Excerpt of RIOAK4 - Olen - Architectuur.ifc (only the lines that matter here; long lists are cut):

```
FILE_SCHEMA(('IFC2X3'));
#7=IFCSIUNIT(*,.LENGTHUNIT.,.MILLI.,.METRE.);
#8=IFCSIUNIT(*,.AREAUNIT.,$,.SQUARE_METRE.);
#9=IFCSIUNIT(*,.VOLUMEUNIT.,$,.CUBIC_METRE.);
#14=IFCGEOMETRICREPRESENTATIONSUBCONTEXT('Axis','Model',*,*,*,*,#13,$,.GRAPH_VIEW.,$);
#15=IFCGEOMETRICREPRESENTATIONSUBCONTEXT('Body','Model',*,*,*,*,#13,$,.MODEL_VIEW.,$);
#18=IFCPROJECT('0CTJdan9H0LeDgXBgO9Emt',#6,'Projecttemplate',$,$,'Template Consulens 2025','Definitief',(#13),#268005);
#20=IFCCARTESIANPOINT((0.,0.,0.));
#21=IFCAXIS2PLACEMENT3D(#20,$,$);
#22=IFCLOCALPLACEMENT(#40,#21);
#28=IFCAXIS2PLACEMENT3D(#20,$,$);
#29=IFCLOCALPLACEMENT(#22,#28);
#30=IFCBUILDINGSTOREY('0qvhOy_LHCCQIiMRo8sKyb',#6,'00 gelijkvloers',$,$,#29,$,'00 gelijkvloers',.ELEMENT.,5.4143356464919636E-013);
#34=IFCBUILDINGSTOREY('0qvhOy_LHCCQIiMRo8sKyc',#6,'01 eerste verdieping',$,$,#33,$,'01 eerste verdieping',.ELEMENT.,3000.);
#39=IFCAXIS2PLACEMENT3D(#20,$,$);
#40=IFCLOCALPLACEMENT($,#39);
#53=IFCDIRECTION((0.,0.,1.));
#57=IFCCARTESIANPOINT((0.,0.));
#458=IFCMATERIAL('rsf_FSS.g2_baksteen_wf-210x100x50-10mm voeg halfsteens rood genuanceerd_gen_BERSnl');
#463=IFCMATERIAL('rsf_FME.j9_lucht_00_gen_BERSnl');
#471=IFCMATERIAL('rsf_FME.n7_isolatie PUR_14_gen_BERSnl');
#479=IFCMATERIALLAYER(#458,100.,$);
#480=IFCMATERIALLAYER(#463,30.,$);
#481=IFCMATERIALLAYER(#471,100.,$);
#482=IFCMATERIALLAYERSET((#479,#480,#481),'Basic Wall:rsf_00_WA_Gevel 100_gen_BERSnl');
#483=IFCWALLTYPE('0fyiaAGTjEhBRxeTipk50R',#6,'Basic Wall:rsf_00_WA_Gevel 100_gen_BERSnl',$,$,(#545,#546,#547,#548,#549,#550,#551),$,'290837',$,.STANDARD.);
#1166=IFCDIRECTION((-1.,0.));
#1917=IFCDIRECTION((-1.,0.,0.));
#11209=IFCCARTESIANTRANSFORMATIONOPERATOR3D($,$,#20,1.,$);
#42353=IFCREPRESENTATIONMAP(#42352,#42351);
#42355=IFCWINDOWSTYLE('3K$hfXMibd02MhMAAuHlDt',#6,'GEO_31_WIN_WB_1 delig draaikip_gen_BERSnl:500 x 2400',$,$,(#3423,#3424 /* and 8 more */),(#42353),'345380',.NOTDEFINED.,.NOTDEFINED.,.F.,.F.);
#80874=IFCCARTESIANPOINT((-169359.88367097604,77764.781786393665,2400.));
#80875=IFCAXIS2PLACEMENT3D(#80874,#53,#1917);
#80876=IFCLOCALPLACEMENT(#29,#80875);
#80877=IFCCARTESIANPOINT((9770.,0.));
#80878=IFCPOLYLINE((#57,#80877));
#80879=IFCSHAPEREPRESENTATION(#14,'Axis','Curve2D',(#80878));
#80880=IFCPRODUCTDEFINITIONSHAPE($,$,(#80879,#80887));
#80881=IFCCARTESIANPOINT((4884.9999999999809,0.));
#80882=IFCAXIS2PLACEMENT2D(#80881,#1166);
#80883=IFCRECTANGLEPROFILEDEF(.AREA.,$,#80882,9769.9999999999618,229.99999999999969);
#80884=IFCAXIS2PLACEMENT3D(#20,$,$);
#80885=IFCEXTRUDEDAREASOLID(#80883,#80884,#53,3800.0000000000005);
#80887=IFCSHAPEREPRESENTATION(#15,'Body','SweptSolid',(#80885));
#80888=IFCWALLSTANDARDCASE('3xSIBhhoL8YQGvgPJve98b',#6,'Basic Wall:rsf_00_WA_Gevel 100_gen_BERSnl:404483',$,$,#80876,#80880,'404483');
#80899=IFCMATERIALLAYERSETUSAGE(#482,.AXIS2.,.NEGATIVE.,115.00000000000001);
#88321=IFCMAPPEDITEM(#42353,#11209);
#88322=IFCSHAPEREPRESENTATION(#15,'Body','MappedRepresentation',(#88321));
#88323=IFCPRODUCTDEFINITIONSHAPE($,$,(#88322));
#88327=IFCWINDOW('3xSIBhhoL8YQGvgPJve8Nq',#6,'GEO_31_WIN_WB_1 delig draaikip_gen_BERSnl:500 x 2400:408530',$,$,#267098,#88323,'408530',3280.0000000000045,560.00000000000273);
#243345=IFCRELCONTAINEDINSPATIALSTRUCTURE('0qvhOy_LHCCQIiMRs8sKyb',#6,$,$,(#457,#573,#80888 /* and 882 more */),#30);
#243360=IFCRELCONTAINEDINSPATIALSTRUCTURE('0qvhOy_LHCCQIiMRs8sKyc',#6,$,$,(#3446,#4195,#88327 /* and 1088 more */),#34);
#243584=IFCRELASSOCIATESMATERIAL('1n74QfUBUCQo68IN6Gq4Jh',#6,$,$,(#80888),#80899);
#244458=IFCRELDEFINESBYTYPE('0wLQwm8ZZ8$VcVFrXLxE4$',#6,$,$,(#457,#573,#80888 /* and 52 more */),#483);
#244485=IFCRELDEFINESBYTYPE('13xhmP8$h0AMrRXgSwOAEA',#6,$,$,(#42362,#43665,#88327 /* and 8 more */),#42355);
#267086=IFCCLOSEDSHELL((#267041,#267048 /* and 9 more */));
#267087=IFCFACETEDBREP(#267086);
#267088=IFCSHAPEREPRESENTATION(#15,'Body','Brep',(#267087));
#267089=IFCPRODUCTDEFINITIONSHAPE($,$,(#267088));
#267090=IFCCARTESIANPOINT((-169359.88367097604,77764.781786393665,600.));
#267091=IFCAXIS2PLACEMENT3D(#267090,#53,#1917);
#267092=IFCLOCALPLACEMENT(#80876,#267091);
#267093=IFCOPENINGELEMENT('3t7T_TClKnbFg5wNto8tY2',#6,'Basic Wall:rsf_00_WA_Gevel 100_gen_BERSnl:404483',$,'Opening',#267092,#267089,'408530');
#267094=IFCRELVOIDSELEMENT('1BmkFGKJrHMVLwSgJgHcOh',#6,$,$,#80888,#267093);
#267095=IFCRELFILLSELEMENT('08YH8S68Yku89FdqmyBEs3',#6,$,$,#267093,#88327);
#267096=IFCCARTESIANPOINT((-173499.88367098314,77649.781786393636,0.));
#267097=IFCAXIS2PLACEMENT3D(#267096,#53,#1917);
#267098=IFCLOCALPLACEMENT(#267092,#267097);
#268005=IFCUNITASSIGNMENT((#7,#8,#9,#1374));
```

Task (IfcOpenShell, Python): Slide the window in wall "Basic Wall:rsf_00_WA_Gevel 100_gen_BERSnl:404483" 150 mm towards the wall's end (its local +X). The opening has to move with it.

```python
import ifcopenshell
import ifcopenshell.api.geometry
import ifcopenshell.util.placement
import ifcopenshell.util.unit

model = ifcopenshell.open("RIOAK4 - Olen - Architectuur.ifc")
unit_scale = ifcopenshell.util.unit.calculate_unit_scale(model)

window = model.by_id(88327)
opening = window.FillsVoids[0].RelatingOpeningElement
wall = opening.VoidsElements[0].RelatingBuildingElement

wall_matrix = ifcopenshell.util.placement.get_local_placement(wall.ObjectPlacement)
shift = wall_matrix[:3, 0] * 0.15 / unit_scale
before = ifcopenshell.util.placement.get_local_placement(window.ObjectPlacement)[:3, 3].copy()

# The window is placed relative to its opening, so it follows when the opening moves.
matrix = ifcopenshell.util.placement.get_local_placement(opening.ObjectPlacement)
matrix[:3, 3] += shift
ifcopenshell.api.geometry.edit_object_placement(
    model, product=opening, matrix=matrix, is_si=False, should_transform_children=True
)

after = ifcopenshell.util.placement.get_local_placement(window.ObjectPlacement)[:3, 3]
print("window moved by", (after - before).round(3) + 0.0)

model.write("RIOAK4 - Olen - Architectuur_v2.ifc")
```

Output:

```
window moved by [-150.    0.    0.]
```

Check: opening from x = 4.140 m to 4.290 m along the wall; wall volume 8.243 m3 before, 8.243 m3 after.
